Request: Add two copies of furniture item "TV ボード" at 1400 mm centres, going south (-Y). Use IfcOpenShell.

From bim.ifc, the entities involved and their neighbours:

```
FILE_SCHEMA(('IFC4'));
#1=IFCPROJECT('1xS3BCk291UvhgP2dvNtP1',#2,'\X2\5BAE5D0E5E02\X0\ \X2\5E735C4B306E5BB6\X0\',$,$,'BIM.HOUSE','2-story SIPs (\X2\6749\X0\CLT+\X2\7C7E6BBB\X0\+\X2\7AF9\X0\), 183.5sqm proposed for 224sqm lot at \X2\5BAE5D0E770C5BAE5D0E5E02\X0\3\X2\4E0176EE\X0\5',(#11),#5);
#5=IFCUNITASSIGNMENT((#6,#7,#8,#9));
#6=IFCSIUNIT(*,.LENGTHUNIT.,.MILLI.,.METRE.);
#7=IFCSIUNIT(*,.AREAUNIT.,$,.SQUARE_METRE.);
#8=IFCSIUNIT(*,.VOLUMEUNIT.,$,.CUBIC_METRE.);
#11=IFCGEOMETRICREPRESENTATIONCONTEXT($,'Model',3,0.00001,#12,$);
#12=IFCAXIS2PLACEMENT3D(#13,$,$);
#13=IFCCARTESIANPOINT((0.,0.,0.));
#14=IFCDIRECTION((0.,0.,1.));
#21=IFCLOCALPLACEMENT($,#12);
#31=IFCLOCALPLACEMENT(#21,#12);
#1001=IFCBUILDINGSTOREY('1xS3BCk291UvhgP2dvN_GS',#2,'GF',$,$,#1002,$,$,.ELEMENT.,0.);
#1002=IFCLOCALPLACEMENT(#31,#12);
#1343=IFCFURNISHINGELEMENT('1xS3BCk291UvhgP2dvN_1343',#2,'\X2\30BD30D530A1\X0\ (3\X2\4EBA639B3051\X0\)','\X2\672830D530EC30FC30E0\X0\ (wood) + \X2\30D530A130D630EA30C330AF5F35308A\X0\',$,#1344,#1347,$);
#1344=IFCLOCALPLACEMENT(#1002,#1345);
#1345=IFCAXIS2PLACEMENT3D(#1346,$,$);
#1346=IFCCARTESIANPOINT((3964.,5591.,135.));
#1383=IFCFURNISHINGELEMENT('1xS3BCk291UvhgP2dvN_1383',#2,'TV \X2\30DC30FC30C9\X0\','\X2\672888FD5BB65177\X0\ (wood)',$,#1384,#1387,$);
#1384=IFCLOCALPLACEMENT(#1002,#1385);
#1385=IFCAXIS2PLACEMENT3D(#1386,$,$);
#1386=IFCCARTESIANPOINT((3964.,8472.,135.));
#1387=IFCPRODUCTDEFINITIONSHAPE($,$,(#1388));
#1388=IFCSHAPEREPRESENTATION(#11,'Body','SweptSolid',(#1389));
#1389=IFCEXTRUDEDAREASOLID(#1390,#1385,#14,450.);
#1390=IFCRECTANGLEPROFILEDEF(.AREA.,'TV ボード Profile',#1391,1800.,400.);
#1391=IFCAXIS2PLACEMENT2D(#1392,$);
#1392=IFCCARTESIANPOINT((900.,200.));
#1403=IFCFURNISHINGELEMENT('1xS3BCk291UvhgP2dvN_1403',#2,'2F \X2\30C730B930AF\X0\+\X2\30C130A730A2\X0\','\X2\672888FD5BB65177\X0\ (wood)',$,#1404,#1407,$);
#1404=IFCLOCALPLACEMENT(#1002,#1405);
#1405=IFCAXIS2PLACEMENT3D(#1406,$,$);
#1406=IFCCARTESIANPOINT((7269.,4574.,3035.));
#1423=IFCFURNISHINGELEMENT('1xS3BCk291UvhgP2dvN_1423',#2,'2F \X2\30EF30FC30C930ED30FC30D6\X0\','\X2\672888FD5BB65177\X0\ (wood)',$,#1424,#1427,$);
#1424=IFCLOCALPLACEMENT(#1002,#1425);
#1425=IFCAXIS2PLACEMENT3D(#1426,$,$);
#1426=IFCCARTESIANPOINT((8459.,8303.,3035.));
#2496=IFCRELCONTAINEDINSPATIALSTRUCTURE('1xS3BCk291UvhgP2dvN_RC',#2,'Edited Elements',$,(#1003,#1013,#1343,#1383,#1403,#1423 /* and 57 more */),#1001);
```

```python
import numpy as np
import ifcopenshell
import ifcopenshell.api.geometry
import ifcopenshell.api.root
import ifcopenshell.util.element
import ifcopenshell.util.placement
import ifcopenshell.util.unit

model = ifcopenshell.open("bim.ifc")
unit_scale = ifcopenshell.util.unit.calculate_unit_scale(model)


def reuse_history(source, copy):
    """copy_class also copies each property set's owner history, people and application; keep the originals."""
    for rel in copy.IsDefinedBy:
        if rel.is_a("IfcRelDefinesByProperties") and (history := rel.RelatingPropertyDefinition.OwnerHistory):
            rel.RelatingPropertyDefinition.OwnerHistory = source.OwnerHistory
            ifcopenshell.util.element.remove_deep2(model, history)


source = model.by_guid("1xS3BCk291UvhgP2dvN_1383")
base = ifcopenshell.util.placement.get_local_placement(source.ObjectPlacement)
step = np.array([0.0, -1.0, 0.0]) * 1.4 / unit_scale

for i in range(1, 3):
    copy = ifcopenshell.api.root.copy_class(model, product=source)
    copy.Representation = ifcopenshell.util.element.copy_deep(
        model, source.Representation, exclude=["IfcGeometricRepresentationContext", "IfcRepresentationMap"]
    )
    reuse_history(source, copy)
    matrix = base.copy()
    matrix[:3, 3] += i * step
    print("added at", matrix[:3, 3].round(3) + 0.0)
    ifcopenshell.api.geometry.edit_object_placement(model, product=copy, matrix=matrix, is_si=False)

model.write("bim_v2.ifc")
```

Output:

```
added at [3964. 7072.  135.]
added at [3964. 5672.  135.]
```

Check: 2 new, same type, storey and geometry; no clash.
